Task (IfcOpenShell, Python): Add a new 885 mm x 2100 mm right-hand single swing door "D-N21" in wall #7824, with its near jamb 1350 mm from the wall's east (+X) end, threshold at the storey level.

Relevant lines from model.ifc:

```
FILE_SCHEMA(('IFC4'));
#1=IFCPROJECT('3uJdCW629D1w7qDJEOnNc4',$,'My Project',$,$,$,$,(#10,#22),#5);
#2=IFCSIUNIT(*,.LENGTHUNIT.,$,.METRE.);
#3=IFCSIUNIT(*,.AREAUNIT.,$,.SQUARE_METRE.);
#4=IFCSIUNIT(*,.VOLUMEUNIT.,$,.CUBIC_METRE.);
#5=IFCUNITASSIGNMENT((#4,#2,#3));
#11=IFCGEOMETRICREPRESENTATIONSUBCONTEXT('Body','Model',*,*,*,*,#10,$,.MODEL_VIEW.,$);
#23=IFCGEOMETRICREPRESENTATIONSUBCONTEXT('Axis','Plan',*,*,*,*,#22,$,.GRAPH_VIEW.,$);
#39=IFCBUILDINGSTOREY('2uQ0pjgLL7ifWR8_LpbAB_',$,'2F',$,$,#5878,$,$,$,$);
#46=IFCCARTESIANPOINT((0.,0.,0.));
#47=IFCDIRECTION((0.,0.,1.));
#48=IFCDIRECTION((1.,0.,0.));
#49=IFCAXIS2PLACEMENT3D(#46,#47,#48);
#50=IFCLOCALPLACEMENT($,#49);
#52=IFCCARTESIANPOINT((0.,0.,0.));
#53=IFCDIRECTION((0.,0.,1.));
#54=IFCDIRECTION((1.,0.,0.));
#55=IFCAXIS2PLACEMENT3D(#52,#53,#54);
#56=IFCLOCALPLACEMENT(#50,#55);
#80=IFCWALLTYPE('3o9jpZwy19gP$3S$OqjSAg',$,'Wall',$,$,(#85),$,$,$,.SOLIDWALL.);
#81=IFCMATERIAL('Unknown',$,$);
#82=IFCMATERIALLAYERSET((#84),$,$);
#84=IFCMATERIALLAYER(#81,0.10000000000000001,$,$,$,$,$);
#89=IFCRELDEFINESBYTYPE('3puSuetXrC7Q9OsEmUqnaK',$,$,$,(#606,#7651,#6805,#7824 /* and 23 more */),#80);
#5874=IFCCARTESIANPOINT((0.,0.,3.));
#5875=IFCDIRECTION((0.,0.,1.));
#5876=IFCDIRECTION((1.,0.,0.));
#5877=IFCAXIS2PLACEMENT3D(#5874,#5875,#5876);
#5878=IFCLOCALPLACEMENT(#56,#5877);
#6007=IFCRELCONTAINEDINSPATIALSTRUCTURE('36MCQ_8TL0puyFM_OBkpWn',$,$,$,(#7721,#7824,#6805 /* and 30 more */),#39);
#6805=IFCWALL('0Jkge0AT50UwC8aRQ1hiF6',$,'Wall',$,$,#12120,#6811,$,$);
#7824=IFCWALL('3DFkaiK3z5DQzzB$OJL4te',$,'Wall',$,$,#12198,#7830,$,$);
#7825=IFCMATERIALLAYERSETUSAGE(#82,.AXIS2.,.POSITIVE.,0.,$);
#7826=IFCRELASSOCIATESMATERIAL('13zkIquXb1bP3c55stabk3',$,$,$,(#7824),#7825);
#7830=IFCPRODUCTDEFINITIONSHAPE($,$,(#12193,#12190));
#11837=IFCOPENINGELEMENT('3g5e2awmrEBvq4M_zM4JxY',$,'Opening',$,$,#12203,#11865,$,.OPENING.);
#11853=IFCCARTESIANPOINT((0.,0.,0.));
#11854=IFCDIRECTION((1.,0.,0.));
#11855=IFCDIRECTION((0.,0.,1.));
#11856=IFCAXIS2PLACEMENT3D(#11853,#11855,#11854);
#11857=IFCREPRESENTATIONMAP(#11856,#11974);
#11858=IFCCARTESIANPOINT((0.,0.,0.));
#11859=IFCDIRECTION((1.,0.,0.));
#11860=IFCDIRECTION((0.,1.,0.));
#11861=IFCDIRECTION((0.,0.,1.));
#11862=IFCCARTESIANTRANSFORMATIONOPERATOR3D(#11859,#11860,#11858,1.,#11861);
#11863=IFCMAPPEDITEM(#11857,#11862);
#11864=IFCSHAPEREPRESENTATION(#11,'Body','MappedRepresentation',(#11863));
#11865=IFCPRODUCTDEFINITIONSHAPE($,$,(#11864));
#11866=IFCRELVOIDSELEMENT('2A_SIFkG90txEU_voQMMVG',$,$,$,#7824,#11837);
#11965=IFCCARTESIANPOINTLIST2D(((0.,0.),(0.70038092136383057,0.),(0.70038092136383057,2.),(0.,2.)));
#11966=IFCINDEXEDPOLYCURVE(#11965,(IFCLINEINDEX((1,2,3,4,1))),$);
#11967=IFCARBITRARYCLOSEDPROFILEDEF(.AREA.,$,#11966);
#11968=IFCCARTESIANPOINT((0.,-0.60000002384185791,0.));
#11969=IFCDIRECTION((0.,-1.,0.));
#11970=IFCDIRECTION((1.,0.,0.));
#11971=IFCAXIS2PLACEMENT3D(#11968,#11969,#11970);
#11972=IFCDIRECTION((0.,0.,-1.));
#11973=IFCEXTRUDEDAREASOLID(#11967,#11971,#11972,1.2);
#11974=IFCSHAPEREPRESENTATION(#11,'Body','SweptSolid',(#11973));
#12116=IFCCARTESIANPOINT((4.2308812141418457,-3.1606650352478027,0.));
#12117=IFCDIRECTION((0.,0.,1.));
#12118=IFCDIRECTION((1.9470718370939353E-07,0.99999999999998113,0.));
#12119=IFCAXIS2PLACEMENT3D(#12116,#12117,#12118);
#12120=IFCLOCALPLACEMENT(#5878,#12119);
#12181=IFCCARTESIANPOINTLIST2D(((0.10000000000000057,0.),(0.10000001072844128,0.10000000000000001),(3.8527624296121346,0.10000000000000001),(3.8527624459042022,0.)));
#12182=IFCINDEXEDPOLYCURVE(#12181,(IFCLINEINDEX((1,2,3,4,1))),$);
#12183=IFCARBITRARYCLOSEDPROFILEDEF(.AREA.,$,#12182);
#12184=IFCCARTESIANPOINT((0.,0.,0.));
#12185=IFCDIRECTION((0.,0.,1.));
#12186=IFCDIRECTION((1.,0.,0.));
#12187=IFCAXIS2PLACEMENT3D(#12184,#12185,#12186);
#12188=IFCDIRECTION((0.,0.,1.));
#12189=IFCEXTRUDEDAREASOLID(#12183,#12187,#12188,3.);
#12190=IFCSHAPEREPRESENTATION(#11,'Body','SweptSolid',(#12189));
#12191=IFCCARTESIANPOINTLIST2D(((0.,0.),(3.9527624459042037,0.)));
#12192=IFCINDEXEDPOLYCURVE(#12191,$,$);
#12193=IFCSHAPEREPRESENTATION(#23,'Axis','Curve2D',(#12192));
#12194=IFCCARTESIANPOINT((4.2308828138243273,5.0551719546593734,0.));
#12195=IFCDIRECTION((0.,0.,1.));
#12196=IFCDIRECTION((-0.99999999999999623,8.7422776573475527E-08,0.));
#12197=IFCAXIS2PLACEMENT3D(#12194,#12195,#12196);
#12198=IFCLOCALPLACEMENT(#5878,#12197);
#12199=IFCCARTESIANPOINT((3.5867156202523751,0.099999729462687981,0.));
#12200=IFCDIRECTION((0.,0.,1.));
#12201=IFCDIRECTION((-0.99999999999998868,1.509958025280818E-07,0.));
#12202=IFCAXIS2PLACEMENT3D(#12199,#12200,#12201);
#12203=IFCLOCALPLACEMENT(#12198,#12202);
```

```python
import numpy as np
import ifcopenshell
import ifcopenshell.api.feature
import ifcopenshell.api.geometry
import ifcopenshell.api.root
import ifcopenshell.api.spatial
import ifcopenshell.geom
import ifcopenshell.util.element
import ifcopenshell.util.placement
import ifcopenshell.util.representation
import ifcopenshell.util.shape
import ifcopenshell.util.unit

model = ifcopenshell.open("model.ifc")
unit_scale = ifcopenshell.util.unit.calculate_unit_scale(model)
settings = ifcopenshell.geom.settings()


def volume(element):
    """Net volume in cubic metres, openings subtracted."""
    shape = ifcopenshell.geom.create_shape(settings, element)
    return ifcopenshell.util.shape.get_volume(shape.geometry)


wall = model.by_id(7824)
storey = ifcopenshell.util.element.get_container(wall, ifc_class="IfcBuildingStorey")
context = ifcopenshell.util.representation.get_context(model, "Model", "Body", "MODEL_VIEW")
before = volume(wall)

width, height, from_end, sill = 0.885, 2.1, 1.35, 0.0  # metres

# The wall runs along its own X axis, and the end named is its -X end.
wall_shape = ifcopenshell.geom.create_shape(settings, wall)
x, y, z = ifcopenshell.util.shape.get_vertices(wall_shape.geometry).T
start = x.min() + from_end
face, thickness = float(y.min()), float(y.max() - y.min())
wall_matrix = ifcopenshell.util.placement.get_local_placement(wall.ObjectPlacement)
level = ifcopenshell.util.placement.get_local_placement(storey.ObjectPlacement)[2, 3]


def in_wall(x, y):
    """Placement at x, y metres in the wall's axes, at sill height."""
    matrix = wall_matrix.copy()
    matrix[:, 3] = wall_matrix @ np.array([x / unit_scale, y / unit_scale, 0.0, 1.0])
    matrix[2, 3] = level + sill / unit_scale
    return matrix


# Opening: a box that overshoots both wall faces by 50 mm.
opening = ifcopenshell.api.root.create_entity(model, ifc_class="IfcOpeningElement", predefined_type="OPENING")
box = ifcopenshell.api.geometry.add_wall_representation(
    model, context=context, length=width, height=height, thickness=thickness + 0.1
)
ifcopenshell.api.geometry.assign_representation(model, product=opening, representation=box)
ifcopenshell.api.geometry.edit_object_placement(model, product=opening, matrix=in_wall(start, face - 0.05), is_si=False)
ifcopenshell.api.feature.add_feature(model, feature=opening, element=wall)

door = ifcopenshell.api.root.create_entity(model, ifc_class="IfcDoor", name="D-N21", predefined_type="DOOR")
door.OverallWidth, door.OverallHeight = width / unit_scale, height / unit_scale
door.OperationType = "SINGLE_SWING_RIGHT"
body = ifcopenshell.api.geometry.add_door_representation(
    model,
    context=context,
    overall_width=door.OverallWidth,
    overall_height=door.OverallHeight,
    operation_type="SINGLE_SWING_RIGHT",
    lining_properties={"LiningDepth": thickness / unit_scale, "ThresholdDepth": thickness / unit_scale},
)
ifcopenshell.api.geometry.assign_representation(model, product=door, representation=body)
ifcopenshell.api.spatial.assign_container(model, products=[door], relating_structure=storey)
ifcopenshell.api.feature.add_filling(model, opening=opening, element=door)

# The lining spans the wall, so the door starts at the wall face.
ifcopenshell.api.geometry.edit_object_placement(model, product=door, matrix=in_wall(start, face), is_si=False)

after = volume(wall)

print(f"wall volume {before:.3f} -> {after:.3f} m3")

model.write("model_updated.ifc")
```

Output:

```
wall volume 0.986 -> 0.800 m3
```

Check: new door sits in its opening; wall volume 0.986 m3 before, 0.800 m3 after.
